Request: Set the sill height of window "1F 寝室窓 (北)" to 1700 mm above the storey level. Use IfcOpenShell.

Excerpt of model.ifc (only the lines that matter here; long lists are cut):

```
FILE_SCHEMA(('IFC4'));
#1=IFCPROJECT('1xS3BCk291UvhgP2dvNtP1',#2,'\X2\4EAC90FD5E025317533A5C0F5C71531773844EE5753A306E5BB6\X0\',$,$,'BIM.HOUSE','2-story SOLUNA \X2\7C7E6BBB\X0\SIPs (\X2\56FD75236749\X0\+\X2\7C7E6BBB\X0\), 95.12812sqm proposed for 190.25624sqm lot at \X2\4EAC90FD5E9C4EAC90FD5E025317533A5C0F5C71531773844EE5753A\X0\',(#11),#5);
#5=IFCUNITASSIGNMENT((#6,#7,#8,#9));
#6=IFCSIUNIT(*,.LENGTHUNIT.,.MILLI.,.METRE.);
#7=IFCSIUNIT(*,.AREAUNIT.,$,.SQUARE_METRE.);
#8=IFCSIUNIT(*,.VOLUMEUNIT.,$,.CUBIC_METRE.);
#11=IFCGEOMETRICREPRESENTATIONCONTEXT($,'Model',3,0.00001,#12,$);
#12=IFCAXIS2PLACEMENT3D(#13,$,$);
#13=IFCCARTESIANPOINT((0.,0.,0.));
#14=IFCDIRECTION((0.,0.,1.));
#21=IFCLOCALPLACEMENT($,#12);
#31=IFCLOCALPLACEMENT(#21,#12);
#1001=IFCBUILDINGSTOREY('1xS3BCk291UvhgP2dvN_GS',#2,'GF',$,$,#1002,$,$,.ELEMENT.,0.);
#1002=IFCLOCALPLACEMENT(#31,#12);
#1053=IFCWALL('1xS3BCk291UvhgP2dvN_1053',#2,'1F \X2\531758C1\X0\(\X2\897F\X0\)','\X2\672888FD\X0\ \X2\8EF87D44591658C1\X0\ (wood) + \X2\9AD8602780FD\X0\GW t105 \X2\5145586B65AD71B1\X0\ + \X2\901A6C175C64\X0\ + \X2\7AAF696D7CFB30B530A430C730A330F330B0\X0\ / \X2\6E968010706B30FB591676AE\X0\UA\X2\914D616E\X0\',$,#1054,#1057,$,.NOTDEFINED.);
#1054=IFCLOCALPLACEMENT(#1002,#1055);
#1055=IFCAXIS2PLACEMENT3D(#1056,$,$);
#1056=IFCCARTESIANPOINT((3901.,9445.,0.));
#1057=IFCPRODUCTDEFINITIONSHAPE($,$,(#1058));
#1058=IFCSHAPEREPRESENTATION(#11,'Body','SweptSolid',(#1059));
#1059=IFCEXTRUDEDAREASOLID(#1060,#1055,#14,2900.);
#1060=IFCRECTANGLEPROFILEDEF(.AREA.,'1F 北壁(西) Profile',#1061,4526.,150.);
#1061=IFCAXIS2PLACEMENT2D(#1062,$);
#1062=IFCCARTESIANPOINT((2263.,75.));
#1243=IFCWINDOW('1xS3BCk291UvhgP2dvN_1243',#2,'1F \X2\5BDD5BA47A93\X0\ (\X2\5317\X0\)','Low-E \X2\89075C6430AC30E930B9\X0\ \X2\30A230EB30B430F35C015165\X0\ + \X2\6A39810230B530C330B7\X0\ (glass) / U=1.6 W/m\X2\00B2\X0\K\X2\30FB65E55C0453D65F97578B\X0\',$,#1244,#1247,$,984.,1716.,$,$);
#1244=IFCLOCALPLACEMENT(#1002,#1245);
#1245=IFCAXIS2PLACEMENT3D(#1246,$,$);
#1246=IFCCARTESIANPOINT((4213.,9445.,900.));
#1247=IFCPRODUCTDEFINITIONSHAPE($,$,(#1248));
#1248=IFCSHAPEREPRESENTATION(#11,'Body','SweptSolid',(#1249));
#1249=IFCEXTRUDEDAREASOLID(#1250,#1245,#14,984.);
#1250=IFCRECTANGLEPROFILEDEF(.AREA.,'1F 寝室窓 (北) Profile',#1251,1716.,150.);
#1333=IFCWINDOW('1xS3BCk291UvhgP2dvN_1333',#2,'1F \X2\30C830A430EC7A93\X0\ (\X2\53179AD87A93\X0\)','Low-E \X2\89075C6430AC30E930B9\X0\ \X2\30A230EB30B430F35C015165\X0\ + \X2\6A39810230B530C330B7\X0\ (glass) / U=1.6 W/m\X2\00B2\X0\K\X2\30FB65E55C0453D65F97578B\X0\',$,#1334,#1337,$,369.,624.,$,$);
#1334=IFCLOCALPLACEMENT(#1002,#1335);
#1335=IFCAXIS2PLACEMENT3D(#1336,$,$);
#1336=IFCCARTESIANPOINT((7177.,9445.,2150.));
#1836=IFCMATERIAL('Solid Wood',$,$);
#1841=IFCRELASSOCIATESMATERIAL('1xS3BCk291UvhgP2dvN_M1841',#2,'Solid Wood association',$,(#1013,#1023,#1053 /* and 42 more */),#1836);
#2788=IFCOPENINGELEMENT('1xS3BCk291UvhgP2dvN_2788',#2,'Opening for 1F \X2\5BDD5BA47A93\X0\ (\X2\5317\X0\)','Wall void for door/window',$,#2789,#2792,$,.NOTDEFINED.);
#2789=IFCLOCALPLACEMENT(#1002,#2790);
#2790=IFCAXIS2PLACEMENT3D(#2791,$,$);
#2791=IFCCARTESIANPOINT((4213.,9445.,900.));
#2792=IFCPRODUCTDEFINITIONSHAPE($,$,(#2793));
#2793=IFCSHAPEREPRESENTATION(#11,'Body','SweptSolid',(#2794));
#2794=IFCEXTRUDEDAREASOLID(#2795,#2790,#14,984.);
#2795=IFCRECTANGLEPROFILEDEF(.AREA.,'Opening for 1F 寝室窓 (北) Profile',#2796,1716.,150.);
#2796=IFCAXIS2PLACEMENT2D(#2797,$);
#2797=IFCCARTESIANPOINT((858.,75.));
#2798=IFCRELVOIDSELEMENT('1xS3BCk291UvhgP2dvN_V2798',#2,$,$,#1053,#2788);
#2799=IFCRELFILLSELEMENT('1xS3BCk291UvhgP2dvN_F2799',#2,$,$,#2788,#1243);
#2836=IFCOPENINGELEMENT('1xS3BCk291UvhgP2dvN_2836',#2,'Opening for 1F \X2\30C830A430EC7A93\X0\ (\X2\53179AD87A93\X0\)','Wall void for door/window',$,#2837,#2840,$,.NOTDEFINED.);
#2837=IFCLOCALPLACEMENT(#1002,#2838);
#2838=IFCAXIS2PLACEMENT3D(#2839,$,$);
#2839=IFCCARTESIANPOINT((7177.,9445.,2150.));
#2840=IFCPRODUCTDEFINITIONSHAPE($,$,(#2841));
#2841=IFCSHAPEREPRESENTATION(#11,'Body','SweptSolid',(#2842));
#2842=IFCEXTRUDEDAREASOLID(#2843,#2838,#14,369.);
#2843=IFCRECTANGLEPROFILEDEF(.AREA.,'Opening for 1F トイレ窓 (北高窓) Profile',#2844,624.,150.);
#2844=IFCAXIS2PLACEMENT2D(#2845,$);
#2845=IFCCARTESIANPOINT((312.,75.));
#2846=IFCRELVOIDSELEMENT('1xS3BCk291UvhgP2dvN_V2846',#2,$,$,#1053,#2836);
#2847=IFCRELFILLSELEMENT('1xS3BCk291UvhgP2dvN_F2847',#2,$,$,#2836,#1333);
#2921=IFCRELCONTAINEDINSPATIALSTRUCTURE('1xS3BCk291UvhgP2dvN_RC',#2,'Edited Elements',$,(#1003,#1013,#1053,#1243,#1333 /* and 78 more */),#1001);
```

```python
import numpy as np
import ifcopenshell
import ifcopenshell.api.geometry
import ifcopenshell.geom
import ifcopenshell.util.element
import ifcopenshell.util.placement
import ifcopenshell.util.shape
import ifcopenshell.util.unit

model = ifcopenshell.open("model.ifc")
unit_scale = ifcopenshell.util.unit.calculate_unit_scale(model)

window = model.by_guid("1xS3BCk291UvhgP2dvN_1243")
opening = window.FillsVoids[0].RelatingOpeningElement
storey = ifcopenshell.util.element.get_container(window, ifc_class="IfcBuildingStorey")
level = ifcopenshell.util.placement.get_local_placement(storey.ObjectPlacement)[2, 3]

# The opening's origin need not be at the sill, so measure its lowest point.
shape = ifcopenshell.geom.create_shape(ifcopenshell.geom.settings(), opening)
bottom = ifcopenshell.util.shape.get_shape_bottom_elevation(shape, shape.geometry) / unit_scale
dz = level + 1700.0 - bottom

shift = np.array([0.0, 0.0, dz])
# The window is not placed relative to its opening, so move both.
for product in (opening, window):
    matrix = ifcopenshell.util.placement.get_local_placement(product.ObjectPlacement)
    matrix[:3, 3] += shift
    ifcopenshell.api.geometry.edit_object_placement(model, product=product, matrix=matrix, is_si=False)

print(f"moved by {dz * unit_scale:+.3f} m")

model.write("model_rev.ifc")
```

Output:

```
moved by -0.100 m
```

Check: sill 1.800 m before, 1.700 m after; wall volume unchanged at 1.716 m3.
